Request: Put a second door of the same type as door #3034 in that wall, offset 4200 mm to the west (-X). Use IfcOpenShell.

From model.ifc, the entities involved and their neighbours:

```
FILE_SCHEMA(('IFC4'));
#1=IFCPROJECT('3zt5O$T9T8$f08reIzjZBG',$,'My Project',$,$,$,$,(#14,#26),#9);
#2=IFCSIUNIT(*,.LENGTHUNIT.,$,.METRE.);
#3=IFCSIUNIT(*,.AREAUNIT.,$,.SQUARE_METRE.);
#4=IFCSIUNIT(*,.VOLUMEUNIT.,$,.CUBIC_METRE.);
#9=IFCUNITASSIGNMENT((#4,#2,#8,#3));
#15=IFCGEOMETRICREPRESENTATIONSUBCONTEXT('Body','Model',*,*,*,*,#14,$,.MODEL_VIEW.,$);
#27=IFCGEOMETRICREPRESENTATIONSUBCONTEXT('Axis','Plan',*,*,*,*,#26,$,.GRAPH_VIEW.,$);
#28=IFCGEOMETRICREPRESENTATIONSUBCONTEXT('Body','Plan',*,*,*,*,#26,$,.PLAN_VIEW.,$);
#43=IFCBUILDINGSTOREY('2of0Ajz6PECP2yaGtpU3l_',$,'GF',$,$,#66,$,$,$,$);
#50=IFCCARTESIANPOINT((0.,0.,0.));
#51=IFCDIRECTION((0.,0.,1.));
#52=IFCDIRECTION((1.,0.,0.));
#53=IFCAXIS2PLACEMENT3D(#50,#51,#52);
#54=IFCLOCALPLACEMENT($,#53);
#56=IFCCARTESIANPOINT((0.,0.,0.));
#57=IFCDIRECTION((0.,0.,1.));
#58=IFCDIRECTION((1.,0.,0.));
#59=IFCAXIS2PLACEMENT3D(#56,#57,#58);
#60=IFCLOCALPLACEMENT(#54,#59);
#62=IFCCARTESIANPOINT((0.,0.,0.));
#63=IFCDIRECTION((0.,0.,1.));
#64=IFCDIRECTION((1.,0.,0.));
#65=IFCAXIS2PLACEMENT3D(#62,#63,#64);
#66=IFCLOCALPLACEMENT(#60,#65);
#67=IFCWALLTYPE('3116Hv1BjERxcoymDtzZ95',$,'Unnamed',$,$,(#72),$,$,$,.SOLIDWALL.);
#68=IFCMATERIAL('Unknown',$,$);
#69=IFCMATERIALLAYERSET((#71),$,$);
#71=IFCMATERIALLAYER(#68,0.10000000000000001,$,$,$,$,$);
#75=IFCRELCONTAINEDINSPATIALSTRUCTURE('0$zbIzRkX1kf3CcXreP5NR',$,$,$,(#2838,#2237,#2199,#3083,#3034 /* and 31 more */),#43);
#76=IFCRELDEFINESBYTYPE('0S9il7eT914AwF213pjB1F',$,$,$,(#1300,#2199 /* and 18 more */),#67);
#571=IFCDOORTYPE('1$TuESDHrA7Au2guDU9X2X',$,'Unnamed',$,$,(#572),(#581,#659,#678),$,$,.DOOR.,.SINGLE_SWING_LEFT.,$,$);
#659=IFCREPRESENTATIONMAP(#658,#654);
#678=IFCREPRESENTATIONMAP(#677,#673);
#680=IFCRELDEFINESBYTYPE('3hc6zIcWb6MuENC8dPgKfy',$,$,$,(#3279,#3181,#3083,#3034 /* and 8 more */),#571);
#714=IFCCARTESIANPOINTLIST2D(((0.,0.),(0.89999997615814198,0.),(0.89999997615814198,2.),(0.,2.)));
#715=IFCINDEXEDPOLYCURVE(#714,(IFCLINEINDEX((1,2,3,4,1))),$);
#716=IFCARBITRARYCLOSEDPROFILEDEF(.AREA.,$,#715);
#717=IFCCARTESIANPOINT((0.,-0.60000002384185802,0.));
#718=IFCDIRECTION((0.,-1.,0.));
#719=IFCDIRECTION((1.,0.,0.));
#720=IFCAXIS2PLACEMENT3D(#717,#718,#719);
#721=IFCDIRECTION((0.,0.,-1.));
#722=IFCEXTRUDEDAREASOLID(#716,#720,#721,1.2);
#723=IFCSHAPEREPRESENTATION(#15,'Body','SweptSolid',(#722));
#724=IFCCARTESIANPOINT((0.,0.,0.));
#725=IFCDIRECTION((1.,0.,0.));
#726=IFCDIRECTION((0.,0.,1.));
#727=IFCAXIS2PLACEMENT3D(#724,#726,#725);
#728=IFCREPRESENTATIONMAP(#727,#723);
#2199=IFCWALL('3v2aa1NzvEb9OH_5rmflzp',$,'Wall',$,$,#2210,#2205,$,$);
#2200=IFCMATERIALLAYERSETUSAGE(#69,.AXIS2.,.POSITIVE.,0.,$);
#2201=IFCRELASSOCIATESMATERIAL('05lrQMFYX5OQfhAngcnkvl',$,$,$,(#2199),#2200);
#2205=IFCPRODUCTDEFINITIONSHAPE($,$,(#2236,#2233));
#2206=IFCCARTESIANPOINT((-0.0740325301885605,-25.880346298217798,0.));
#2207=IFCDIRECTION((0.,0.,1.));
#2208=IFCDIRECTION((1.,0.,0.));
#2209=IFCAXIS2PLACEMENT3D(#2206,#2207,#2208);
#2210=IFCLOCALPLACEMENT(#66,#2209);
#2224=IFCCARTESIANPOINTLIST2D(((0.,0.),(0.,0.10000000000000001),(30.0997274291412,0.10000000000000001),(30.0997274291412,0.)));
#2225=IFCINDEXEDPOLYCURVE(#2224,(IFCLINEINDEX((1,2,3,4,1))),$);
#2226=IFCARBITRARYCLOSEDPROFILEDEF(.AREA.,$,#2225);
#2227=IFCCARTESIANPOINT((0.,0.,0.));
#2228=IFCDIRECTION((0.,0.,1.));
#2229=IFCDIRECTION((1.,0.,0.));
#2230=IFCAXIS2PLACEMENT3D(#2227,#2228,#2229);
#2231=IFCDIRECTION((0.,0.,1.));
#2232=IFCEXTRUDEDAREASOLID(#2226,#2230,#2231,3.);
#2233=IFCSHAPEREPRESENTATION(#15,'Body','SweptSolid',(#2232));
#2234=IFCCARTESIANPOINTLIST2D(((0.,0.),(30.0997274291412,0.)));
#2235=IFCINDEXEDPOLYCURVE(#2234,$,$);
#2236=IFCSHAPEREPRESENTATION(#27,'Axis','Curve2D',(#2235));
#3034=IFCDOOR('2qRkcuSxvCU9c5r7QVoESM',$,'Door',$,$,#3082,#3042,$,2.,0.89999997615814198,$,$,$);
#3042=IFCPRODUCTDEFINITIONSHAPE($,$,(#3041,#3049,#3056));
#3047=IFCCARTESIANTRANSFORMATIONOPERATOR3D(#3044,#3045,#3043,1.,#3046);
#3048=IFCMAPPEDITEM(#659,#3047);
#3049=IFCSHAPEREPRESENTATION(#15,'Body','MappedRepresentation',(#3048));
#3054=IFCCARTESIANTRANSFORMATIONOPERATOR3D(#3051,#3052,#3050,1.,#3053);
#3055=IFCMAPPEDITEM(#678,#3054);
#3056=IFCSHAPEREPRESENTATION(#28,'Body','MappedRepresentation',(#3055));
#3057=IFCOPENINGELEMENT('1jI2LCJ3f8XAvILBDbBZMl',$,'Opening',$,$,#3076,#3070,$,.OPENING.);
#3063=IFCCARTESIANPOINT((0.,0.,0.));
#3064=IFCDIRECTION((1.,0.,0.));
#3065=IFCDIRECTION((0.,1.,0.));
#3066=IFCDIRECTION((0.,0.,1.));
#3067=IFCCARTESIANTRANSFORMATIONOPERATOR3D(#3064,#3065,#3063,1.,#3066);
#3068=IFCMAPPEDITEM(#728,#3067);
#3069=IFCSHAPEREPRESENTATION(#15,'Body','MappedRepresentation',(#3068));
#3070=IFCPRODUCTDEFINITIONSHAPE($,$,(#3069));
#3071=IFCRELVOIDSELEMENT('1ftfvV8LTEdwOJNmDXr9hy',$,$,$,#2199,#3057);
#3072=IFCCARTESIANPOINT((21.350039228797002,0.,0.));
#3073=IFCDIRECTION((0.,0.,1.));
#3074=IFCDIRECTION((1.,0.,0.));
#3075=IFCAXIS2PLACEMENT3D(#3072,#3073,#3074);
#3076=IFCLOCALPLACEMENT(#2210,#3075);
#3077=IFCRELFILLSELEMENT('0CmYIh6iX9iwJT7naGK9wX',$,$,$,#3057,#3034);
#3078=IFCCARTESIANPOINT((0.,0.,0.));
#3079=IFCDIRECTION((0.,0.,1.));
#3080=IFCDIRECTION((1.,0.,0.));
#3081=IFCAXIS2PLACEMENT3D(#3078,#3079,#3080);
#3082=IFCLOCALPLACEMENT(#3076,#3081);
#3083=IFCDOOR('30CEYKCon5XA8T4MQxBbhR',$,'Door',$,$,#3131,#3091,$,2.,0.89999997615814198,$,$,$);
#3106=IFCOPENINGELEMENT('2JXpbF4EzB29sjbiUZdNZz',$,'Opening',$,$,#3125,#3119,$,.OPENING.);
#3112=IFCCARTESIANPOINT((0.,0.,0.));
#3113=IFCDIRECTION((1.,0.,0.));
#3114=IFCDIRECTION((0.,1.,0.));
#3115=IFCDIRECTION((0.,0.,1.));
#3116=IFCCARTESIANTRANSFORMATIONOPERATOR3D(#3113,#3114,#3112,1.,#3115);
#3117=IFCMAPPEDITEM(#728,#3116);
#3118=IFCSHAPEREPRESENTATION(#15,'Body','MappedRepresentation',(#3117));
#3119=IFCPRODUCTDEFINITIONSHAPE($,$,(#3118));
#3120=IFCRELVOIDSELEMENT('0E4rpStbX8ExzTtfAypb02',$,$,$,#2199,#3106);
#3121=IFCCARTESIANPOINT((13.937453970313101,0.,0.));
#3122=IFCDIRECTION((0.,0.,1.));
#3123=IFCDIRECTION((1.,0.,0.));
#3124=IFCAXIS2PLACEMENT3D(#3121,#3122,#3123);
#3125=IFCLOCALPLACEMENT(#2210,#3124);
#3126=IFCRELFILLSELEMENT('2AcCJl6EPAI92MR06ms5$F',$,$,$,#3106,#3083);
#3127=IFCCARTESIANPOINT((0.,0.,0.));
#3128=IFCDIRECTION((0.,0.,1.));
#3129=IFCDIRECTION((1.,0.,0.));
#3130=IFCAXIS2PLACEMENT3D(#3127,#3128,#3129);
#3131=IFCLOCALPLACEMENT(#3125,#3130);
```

```python
import ifcopenshell
import ifcopenshell.api.feature
import ifcopenshell.api.geometry
import ifcopenshell.api.root
import ifcopenshell.geom
import ifcopenshell.util.element
import ifcopenshell.util.placement
import ifcopenshell.util.shape
import ifcopenshell.util.unit

model = ifcopenshell.open("model.ifc")
unit_scale = ifcopenshell.util.unit.calculate_unit_scale(model)
settings = ifcopenshell.geom.settings()


def volume(element):
    """Net volume in cubic metres, openings subtracted."""
    shape = ifcopenshell.geom.create_shape(settings, element)
    return ifcopenshell.util.shape.get_volume(shape.geometry)


door = model.by_guid("2qRkcuSxvCU9c5r7QVoESM")
opening = door.FillsVoids[0].RelatingOpeningElement
wall = opening.VoidsElements[0].RelatingBuildingElement
before = volume(wall)
shift = ifcopenshell.util.placement.get_local_placement(wall.ObjectPlacement)[:3, 0] * -4.2 / unit_scale

# copy_class copies the void relationship, type, container and properties, but no geometry.
new_opening = ifcopenshell.api.root.copy_class(model, product=opening)
new_opening.Representation = ifcopenshell.util.element.copy_deep(
    model, opening.Representation, exclude=["IfcGeometricRepresentationContext", "IfcRepresentationMap"]
)
new_door = ifcopenshell.api.root.copy_class(model, product=door)
new_door.Representation = ifcopenshell.util.element.copy_deep(
    model, door.Representation, exclude=["IfcGeometricRepresentationContext", "IfcRepresentationMap"]
)
ifcopenshell.api.feature.add_filling(model, opening=new_opening, element=new_door)

for old, new in ((opening, new_opening), (door, new_door)):
    matrix = ifcopenshell.util.placement.get_local_placement(old.ObjectPlacement)
    matrix[:3, 3] += shift
    ifcopenshell.api.geometry.edit_object_placement(model, product=new, matrix=matrix, is_si=False)

after = volume(wall)

print(f"wall volume {before:.3f} -> {after:.3f} m3")

model.write("model_updated.ifc")
```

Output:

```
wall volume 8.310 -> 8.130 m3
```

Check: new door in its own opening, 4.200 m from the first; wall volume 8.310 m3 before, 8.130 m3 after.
